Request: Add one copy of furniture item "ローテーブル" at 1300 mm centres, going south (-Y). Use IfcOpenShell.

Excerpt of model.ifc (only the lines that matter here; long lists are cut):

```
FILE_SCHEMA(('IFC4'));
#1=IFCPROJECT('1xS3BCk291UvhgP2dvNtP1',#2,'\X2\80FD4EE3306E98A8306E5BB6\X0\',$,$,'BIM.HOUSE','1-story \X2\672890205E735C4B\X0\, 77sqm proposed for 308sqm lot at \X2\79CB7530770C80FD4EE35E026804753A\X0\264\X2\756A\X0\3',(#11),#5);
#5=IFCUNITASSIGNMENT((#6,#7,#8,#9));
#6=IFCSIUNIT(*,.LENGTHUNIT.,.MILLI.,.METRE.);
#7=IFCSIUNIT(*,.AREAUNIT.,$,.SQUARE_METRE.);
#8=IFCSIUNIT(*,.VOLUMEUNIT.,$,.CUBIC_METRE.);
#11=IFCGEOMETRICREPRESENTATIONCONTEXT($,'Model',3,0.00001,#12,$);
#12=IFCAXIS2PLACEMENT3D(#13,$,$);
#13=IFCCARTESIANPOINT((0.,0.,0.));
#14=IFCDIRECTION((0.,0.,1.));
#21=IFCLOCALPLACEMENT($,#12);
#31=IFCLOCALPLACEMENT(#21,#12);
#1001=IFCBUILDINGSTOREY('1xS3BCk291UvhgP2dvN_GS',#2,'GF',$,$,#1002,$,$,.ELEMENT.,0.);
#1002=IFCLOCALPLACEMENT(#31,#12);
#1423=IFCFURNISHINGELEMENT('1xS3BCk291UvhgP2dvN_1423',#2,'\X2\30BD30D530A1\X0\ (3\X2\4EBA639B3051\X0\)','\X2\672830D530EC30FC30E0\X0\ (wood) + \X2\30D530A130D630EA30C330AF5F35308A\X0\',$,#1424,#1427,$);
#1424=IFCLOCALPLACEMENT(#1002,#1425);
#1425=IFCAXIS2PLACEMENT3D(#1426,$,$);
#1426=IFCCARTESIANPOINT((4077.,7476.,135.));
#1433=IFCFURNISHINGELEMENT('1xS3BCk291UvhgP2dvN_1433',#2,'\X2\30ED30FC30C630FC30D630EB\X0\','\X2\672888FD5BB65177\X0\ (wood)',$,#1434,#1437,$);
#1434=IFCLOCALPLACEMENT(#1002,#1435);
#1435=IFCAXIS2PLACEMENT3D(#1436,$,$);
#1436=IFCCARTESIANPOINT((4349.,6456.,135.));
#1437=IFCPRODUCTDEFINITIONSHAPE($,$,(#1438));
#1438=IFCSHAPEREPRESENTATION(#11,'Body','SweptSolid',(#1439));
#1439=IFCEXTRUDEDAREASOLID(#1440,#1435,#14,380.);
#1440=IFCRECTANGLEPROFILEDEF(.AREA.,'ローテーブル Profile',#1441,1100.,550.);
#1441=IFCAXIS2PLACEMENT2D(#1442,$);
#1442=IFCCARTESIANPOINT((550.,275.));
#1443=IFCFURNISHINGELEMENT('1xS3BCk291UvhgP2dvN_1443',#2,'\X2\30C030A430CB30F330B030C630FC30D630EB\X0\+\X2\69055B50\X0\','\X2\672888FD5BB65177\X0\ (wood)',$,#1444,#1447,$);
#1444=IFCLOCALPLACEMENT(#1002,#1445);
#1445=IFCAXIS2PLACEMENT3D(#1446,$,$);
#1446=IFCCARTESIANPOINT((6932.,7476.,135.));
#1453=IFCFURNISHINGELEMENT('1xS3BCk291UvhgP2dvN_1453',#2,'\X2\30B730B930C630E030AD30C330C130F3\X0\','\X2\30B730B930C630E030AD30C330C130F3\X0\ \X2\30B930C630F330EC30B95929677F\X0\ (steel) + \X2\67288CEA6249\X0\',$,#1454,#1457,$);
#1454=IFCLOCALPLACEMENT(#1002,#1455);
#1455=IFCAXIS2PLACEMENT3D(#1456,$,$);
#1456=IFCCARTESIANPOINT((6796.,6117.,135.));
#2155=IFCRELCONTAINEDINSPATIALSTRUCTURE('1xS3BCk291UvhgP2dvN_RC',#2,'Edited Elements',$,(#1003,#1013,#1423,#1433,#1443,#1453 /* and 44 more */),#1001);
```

```python
import numpy as np
import ifcopenshell
import ifcopenshell.api.geometry
import ifcopenshell.api.root
import ifcopenshell.util.element
import ifcopenshell.util.placement

model = ifcopenshell.open("model.ifc")


def reuse_history(source, copy):
    """copy_class also copies each property set's owner history, people and application; keep the originals."""
    for rel in copy.IsDefinedBy:
        if rel.is_a("IfcRelDefinesByProperties") and (history := rel.RelatingPropertyDefinition.OwnerHistory):
            rel.RelatingPropertyDefinition.OwnerHistory = source.OwnerHistory
            ifcopenshell.util.element.remove_deep2(model, history)


source = model.by_guid("1xS3BCk291UvhgP2dvN_1433")
base = ifcopenshell.util.placement.get_local_placement(source.ObjectPlacement)
step = np.array([0.0, -1.0, 0.0]) * 1300.0

for i in range(1, 2):
    copy = ifcopenshell.api.root.copy_class(model, product=source)
    copy.Representation = ifcopenshell.util.element.copy_deep(
        model, source.Representation, exclude=["IfcGeometricRepresentationContext", "IfcRepresentationMap"]
    )
    reuse_history(source, copy)
    matrix = base.copy()
    matrix[:3, 3] += i * step
    print("added at", matrix[:3, 3].round(3) + 0.0)
    ifcopenshell.api.geometry.edit_object_placement(model, product=copy, matrix=matrix, is_si=False)

model.write("model_edited.ifc")
```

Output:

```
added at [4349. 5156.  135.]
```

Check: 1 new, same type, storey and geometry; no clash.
